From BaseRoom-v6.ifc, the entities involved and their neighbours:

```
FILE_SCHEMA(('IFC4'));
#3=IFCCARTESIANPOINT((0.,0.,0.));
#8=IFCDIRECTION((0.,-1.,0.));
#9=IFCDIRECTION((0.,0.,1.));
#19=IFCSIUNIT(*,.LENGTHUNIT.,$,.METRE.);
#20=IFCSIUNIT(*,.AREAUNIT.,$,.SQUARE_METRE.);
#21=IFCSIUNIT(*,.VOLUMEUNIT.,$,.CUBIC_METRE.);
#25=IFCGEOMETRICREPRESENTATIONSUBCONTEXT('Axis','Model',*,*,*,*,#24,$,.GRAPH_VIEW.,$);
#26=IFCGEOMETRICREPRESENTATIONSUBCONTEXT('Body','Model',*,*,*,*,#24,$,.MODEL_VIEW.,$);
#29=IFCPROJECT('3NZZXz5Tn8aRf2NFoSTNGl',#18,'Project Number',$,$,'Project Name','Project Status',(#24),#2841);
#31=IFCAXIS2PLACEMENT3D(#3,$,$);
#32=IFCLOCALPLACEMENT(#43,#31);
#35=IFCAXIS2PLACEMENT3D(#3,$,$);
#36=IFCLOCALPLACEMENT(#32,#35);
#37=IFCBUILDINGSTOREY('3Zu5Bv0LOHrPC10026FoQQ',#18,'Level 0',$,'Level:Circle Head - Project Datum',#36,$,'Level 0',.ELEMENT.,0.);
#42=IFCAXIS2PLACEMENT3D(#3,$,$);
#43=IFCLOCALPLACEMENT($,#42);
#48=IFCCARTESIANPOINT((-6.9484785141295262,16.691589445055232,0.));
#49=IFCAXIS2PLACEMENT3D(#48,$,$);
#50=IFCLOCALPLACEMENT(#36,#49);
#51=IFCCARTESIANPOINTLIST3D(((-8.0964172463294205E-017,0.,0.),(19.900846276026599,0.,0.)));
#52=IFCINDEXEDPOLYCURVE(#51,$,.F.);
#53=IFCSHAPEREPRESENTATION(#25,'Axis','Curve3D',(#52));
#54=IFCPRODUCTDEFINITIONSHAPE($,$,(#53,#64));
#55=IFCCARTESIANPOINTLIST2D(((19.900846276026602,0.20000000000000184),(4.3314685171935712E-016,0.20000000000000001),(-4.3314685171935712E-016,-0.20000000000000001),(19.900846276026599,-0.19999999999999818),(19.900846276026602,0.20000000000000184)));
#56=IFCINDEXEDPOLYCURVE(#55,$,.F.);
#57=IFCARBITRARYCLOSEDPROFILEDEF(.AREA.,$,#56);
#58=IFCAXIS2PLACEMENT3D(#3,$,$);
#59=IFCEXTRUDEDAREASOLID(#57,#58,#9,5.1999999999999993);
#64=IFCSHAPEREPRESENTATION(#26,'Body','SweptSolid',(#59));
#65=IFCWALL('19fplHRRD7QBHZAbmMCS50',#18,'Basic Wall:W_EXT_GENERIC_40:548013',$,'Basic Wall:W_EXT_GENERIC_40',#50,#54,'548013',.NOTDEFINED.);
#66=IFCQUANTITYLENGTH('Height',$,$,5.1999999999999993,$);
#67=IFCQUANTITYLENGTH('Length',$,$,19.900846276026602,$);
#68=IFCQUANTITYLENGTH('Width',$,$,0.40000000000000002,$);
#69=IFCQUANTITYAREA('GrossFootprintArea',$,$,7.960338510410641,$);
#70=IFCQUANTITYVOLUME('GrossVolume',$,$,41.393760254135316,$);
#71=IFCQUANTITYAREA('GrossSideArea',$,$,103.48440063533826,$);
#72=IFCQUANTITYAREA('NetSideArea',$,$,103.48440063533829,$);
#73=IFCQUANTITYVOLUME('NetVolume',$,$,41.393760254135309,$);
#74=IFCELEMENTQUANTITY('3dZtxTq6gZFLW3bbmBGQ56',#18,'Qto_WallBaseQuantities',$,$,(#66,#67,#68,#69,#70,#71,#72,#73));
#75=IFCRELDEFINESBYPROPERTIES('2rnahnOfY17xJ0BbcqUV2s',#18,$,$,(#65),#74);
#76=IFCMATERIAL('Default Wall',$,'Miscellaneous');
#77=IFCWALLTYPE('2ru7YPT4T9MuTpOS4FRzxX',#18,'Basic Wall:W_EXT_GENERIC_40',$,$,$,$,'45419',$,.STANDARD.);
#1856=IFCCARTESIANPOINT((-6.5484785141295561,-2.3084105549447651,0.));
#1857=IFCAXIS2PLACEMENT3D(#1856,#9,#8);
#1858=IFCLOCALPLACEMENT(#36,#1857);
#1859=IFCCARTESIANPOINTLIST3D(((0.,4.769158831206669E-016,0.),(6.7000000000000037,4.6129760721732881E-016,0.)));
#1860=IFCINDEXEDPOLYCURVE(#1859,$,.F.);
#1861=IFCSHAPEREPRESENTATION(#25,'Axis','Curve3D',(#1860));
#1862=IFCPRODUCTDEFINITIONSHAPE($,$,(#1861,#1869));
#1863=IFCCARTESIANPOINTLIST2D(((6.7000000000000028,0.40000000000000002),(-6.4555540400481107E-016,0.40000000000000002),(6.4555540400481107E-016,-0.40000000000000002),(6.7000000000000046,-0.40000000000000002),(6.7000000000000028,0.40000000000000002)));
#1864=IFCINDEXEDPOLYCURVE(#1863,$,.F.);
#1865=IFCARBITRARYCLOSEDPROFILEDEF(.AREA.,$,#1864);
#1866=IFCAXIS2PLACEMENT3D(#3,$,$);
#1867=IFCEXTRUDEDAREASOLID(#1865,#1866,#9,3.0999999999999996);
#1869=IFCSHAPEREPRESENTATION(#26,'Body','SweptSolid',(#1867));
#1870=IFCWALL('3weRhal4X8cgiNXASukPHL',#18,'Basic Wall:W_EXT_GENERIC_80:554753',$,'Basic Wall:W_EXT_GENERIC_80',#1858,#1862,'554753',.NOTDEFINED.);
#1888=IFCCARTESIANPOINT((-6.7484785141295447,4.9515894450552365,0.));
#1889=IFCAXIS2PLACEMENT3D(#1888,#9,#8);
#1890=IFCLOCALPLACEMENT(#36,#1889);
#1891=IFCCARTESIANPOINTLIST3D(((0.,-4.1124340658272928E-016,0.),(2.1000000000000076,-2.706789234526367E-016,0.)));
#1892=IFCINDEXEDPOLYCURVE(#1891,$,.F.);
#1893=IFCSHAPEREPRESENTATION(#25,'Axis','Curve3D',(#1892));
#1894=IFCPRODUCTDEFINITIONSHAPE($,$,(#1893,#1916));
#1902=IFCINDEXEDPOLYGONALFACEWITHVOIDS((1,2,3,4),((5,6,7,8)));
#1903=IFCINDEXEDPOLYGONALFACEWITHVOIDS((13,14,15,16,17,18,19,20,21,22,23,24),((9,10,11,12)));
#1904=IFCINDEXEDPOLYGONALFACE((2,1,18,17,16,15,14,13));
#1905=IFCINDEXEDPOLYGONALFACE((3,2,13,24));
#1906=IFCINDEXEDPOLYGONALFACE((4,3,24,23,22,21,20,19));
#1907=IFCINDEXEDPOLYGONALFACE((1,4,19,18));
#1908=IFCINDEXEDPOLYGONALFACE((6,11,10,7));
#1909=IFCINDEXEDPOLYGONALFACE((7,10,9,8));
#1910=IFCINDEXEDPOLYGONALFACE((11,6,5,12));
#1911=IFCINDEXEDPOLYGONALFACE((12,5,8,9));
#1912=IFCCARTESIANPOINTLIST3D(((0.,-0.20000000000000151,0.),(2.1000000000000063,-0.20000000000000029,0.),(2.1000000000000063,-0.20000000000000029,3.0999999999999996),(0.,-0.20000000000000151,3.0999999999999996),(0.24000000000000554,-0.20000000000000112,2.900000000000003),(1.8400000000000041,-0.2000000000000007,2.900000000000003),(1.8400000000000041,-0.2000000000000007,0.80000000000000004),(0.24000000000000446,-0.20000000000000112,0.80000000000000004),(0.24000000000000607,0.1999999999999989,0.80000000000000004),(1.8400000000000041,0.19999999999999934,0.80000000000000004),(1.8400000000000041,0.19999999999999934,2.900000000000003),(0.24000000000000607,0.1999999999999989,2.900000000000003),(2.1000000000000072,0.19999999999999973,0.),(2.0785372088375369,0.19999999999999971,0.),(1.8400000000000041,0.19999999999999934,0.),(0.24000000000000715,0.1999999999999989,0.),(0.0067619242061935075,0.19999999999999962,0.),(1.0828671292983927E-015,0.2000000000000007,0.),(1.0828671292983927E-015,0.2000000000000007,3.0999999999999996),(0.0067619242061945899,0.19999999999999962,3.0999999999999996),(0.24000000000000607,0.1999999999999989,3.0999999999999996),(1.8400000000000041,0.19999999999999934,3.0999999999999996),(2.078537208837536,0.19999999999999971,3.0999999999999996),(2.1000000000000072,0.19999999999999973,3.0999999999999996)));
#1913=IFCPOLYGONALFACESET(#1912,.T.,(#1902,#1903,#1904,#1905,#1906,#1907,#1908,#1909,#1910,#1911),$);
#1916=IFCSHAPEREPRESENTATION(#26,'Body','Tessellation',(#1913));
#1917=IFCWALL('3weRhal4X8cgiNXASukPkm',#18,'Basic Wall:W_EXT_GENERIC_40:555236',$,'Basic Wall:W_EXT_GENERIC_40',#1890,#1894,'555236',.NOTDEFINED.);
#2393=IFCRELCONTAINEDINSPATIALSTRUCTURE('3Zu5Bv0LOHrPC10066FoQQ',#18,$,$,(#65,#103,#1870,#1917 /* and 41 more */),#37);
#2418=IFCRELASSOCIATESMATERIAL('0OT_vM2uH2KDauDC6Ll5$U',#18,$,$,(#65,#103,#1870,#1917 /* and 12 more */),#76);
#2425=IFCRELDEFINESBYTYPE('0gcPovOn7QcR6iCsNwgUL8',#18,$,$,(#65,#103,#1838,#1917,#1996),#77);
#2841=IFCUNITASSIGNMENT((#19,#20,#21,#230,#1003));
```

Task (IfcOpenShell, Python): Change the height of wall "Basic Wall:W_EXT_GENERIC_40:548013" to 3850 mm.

```python
import ifcopenshell
import ifcopenshell.api.pset
import ifcopenshell.geom
import ifcopenshell.util.element
import ifcopenshell.util.representation
import ifcopenshell.util.shape
import ifcopenshell.util.unit

model = ifcopenshell.open("BaseRoom-v6.ifc")
unit_scale = ifcopenshell.util.unit.calculate_unit_scale(model)
area_scale = ifcopenshell.util.unit.calculate_unit_scale(model, "AREAUNIT")
volume_scale = ifcopenshell.util.unit.calculate_unit_scale(model, "VOLUMEUNIT")
settings = ifcopenshell.geom.settings()


def volume(element):
    """Net volume in cubic metres, openings subtracted."""
    shape = ifcopenshell.geom.create_shape(settings, element)
    return ifcopenshell.util.shape.get_volume(shape.geometry)


wall = model.by_guid("19fplHRRD7QBHZAbmMCS50")
before = volume(wall)

body = ifcopenshell.util.representation.get_representation(wall, "Model", "Body")
solid = body.Items[0]
old_height = solid.Depth
solid.Depth = 3.85
after = volume(wall)
thickness = 0.4  # wall thickness in metres

# Update the stored height, areas and volumes.
qto = model.by_id(ifcopenshell.util.element.get_pset(wall, "Qto_WallBaseQuantities", should_inherit=False)["id"])
ifcopenshell.api.pset.edit_qto(model, qto=qto, properties={
    "Height": solid.Depth,
    "GrossVolume": ifcopenshell.util.element.get_pset(wall, "Qto_WallBaseQuantities", "GrossVolume") * solid.Depth / old_height,
    "GrossSideArea": ifcopenshell.util.element.get_pset(wall, "Qto_WallBaseQuantities", "GrossSideArea") * solid.Depth / old_height,
    "NetSideArea": after / thickness / area_scale,
    "NetVolume": after / volume_scale,
})

print(f"height {old_height:g} -> {solid.Depth:g}, volume {before:.3f} -> {after:.3f} m3")

model.write("BaseRoom-v6_v2.ifc")
```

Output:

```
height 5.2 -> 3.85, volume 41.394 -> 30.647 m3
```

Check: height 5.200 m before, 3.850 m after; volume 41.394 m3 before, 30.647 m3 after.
